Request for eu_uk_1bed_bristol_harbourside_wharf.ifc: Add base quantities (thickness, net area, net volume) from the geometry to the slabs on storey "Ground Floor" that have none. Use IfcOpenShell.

First a look at what the model holds.

```python
import ifcopenshell
import ifcopenshell.util.element
import ifcopenshell.util.unit

model = ifcopenshell.open("eu_uk_1bed_bristol_harbourside_wharf.ifc")
print(model.schema)
for unit_type in ("LENGTHUNIT", "AREAUNIT", "VOLUMEUNIT"):
    print(unit_type, ifcopenshell.util.unit.calculate_unit_scale(model, unit_type))
storey = next(s for s in model.by_type("IfcBuildingStorey") if s.Name == "Ground Floor")
slabs = [e for e in ifcopenshell.util.element.get_decomposition(storey) if e.is_a("IfcSlab")]
for e in sorted(slabs, key=lambda e: e.id()):
    print(e.id(), e.is_a(), e.Name, list(ifcopenshell.util.element.get_psets(e, qtos_only=True)), sep=" | ")
```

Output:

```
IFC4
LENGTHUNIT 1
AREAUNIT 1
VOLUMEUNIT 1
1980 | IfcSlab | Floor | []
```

```python
import ifcopenshell
import ifcopenshell.api.pset
import ifcopenshell.geom
import ifcopenshell.util.element
import ifcopenshell.util.shape
import ifcopenshell.util.unit

model = ifcopenshell.open("eu_uk_1bed_bristol_harbourside_wharf.ifc")
unit_scale = ifcopenshell.util.unit.calculate_unit_scale(model)
area_scale = ifcopenshell.util.unit.calculate_unit_scale(model, "AREAUNIT")
volume_scale = ifcopenshell.util.unit.calculate_unit_scale(model, "VOLUMEUNIT")
settings = ifcopenshell.geom.settings()

storey = next(s for s in model.by_type("IfcBuildingStorey") if s.Name == "Ground Floor")
slabs = [e for e in ifcopenshell.util.element.get_decomposition(storey) if e.is_a("IfcSlab")]

for e in sorted(slabs, key=lambda e: e.id()):
    if ifcopenshell.util.element.get_psets(e, qtos_only=True, should_inherit=False):
        continue
    # Geometry comes back in metres, in the element's own axes.
    shape = ifcopenshell.geom.create_shape(settings, e)
    values = {
        "Width": ifcopenshell.util.shape.get_z(shape.geometry) / unit_scale,
        "NetArea": ifcopenshell.util.shape.get_footprint_area(shape.geometry) / area_scale,
        "NetVolume": ifcopenshell.util.shape.get_volume(shape.geometry) / volume_scale,
    }
    qto = ifcopenshell.api.pset.add_qto(model, product=e, name="Qto_SlabBaseQuantities")
    ifcopenshell.api.pset.edit_qto(model, qto=qto, properties=values)
    print(e.id(), {k: round(v, 3) for k, v in values.items()})

model.write("eu_uk_1bed_bristol_harbourside_wharf_updated.ifc")
```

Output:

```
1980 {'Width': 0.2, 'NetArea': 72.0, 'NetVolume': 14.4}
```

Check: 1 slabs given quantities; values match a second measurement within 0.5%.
